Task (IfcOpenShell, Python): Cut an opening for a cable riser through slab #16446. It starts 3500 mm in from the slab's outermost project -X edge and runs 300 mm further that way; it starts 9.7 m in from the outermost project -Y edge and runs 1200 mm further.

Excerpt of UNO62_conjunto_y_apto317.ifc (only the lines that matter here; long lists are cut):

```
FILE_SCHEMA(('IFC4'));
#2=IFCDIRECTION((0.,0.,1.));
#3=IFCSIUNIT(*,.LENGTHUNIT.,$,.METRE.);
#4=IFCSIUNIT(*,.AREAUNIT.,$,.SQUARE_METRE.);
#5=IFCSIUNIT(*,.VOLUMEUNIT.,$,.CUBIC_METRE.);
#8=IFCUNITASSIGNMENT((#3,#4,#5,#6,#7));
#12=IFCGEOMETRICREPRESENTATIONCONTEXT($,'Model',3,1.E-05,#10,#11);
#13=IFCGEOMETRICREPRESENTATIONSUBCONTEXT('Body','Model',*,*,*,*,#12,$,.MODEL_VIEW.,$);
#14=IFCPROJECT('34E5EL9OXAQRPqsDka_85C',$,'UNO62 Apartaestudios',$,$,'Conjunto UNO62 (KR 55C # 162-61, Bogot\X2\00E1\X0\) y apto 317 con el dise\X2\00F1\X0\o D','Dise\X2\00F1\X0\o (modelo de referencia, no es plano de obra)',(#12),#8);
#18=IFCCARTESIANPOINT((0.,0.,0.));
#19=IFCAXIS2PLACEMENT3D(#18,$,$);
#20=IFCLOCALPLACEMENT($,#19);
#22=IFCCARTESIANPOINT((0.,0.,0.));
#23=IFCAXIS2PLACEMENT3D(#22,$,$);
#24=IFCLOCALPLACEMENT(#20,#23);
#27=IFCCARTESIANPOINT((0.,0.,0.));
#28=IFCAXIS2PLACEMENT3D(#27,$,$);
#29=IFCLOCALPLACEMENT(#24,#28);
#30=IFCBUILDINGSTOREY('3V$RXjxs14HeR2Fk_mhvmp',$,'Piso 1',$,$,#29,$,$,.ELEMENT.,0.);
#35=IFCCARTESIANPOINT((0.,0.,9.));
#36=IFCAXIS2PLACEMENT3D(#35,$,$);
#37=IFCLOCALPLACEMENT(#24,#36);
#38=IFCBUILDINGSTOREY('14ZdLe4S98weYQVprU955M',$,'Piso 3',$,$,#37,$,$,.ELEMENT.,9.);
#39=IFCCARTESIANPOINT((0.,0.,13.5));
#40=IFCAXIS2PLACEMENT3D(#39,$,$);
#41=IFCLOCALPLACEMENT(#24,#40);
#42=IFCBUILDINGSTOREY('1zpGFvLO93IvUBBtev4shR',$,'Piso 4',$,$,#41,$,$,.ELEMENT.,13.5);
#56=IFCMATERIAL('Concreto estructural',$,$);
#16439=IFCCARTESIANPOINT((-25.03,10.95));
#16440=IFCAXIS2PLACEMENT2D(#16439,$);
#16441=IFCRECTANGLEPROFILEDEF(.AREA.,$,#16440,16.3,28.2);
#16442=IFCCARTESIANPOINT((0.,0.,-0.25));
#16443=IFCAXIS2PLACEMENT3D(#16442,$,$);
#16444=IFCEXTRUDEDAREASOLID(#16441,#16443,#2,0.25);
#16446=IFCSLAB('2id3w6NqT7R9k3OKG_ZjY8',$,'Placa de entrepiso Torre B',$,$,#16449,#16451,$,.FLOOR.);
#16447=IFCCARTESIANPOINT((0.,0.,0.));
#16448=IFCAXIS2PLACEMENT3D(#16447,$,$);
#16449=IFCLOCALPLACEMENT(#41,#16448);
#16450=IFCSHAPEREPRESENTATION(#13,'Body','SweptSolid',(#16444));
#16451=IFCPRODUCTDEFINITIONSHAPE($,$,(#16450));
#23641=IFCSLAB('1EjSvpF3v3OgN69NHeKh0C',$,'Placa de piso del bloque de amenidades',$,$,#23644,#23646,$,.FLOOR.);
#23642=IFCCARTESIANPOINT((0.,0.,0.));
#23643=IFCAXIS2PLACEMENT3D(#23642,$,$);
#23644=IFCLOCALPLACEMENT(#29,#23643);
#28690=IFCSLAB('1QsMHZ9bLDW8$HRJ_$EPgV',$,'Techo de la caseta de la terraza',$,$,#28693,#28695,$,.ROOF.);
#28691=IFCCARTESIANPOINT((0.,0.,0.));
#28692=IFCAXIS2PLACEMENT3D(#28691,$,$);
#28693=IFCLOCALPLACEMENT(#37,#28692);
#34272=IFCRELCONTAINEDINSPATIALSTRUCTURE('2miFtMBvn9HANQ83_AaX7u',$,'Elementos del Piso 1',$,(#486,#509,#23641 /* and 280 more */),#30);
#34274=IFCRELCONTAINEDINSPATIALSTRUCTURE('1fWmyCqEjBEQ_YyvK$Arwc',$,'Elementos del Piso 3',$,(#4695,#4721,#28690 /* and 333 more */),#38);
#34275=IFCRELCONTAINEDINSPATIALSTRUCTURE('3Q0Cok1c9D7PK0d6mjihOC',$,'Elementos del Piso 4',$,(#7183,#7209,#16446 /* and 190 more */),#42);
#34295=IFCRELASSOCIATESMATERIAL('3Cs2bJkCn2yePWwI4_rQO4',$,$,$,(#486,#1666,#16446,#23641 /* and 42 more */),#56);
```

```python
import numpy as np
import ifcopenshell
import ifcopenshell.api.feature
import ifcopenshell.api.geometry
import ifcopenshell.api.root
import ifcopenshell.geom
import ifcopenshell.util.placement
import ifcopenshell.util.representation
import ifcopenshell.util.shape
import ifcopenshell.util.unit

model = ifcopenshell.open("UNO62_conjunto_y_apto317.ifc")
unit_scale = ifcopenshell.util.unit.calculate_unit_scale(model)
settings = ifcopenshell.geom.settings()


def volume(element):
    """Net volume in cubic metres, openings subtracted."""
    shape = ifcopenshell.geom.create_shape(settings, element)
    return ifcopenshell.util.shape.get_volume(shape.geometry)


slab = model.by_id(16446)
before = volume(slab)

# Extent in the slab's own axes, in metres. The edges named are its -X and -Y sides.
slab_shape = ifcopenshell.geom.create_shape(settings, slab)
vertices = ifcopenshell.util.shape.get_vertices(slab_shape.geometry)
x_min, y_min, bottom = vertices.min(axis=0)
top = vertices[:, 2].max()

opening = ifcopenshell.api.root.create_entity(model, ifc_class="IfcOpeningElement", name="Cable riser opening", predefined_type="OPENING")
context = ifcopenshell.util.representation.get_context(model, "Model", "Body", "MODEL_VIEW")
width, depth = 0.3, 1.2
outline = [(0.0, 0.0), (width, 0.0), (width, depth), (0.0, depth), (0.0, 0.0)]
# Overshoot both faces by 50 mm so the cut is clean.
shape = ifcopenshell.api.geometry.add_slab_representation(
    model, context=context, depth=top - bottom + 0.1, polyline=outline
)
ifcopenshell.api.geometry.assign_representation(model, product=opening, representation=shape)

matrix = ifcopenshell.util.placement.get_local_placement(slab.ObjectPlacement)
matrix[:, 3] = matrix @ np.append(np.array([x_min + 3.5, y_min + 9.7, bottom - 0.05]) / unit_scale, 1.0)
ifcopenshell.api.geometry.edit_object_placement(model, product=opening, matrix=matrix, is_si=False)
ifcopenshell.api.feature.add_feature(model, feature=opening, element=slab)

after = volume(slab)

print(f"slab volume {before:.3f} -> {after:.3f} m3")

model.write("UNO62_conjunto_y_apto317_rev.ifc")
```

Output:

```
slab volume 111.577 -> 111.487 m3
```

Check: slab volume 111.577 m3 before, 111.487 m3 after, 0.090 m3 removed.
